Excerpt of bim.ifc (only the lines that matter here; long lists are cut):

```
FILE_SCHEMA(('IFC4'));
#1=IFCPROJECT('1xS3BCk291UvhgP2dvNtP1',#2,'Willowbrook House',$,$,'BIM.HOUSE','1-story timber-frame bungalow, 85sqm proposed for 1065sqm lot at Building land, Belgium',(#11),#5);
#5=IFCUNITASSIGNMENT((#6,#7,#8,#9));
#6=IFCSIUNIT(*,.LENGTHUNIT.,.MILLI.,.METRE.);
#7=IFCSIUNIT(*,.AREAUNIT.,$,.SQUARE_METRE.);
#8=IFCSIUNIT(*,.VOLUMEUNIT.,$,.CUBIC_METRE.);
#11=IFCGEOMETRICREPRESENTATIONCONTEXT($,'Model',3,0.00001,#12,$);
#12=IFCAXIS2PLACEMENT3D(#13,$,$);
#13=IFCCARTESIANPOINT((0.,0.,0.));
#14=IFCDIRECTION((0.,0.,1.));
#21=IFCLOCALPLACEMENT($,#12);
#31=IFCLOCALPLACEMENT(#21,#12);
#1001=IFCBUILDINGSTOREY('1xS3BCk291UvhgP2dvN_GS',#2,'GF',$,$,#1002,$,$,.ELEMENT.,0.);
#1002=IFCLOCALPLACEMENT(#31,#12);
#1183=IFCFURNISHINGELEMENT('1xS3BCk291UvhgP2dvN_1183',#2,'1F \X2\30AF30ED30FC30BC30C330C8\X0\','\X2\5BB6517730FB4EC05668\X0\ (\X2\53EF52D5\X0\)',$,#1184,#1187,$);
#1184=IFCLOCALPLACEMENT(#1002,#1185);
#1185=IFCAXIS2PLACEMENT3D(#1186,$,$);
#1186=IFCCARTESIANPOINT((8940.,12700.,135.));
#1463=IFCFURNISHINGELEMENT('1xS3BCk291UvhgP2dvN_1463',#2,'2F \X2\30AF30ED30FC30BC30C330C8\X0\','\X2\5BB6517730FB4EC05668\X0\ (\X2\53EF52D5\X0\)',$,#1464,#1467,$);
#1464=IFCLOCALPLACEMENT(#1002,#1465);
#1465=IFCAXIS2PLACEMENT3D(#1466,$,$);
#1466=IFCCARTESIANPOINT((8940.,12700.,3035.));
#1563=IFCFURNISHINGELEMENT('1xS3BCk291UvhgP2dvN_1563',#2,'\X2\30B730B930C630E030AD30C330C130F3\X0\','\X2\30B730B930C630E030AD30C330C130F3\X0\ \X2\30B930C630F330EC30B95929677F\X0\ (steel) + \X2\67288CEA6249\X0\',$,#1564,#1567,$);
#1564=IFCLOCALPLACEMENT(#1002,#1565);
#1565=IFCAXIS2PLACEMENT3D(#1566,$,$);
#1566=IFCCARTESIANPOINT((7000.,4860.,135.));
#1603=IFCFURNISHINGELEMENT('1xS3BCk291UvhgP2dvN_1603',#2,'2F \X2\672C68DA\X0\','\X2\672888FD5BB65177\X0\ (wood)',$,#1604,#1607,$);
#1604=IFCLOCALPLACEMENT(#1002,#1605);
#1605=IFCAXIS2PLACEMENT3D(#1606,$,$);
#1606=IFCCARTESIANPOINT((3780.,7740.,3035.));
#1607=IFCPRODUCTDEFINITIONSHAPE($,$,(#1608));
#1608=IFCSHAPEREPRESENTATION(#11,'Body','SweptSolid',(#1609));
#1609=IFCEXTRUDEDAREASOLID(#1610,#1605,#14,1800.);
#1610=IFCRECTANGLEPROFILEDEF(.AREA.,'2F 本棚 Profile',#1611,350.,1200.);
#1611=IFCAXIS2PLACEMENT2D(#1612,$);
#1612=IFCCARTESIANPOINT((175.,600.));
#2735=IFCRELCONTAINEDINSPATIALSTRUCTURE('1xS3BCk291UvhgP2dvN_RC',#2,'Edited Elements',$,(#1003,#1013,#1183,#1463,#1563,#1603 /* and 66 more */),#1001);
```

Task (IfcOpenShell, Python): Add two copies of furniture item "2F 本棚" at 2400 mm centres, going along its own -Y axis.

```python
import ifcopenshell
import ifcopenshell.api.geometry
import ifcopenshell.api.root
import ifcopenshell.util.element
import ifcopenshell.util.placement
import ifcopenshell.util.unit

model = ifcopenshell.open("bim.ifc")
unit_scale = ifcopenshell.util.unit.calculate_unit_scale(model)


def reuse_history(source, copy):
    """copy_class also copies each property set's owner history, people and application; keep the originals."""
    for rel in copy.IsDefinedBy:
        if rel.is_a("IfcRelDefinesByProperties") and (history := rel.RelatingPropertyDefinition.OwnerHistory):
            rel.RelatingPropertyDefinition.OwnerHistory = source.OwnerHistory
            ifcopenshell.util.element.remove_deep2(model, history)


source = model.by_guid("1xS3BCk291UvhgP2dvN_1603")
base = ifcopenshell.util.placement.get_local_placement(source.ObjectPlacement)
step = -base[:3, 1] * 2.4 / unit_scale

for i in range(1, 3):
    copy = ifcopenshell.api.root.copy_class(model, product=source)
    copy.Representation = ifcopenshell.util.element.copy_deep(
        model, source.Representation, exclude=["IfcGeometricRepresentationContext", "IfcRepresentationMap"]
    )
    reuse_history(source, copy)
    matrix = base.copy()
    matrix[:3, 3] += i * step
    print("added at", matrix[:3, 3].round(3) + 0.0)
    ifcopenshell.api.geometry.edit_object_placement(model, product=copy, matrix=matrix, is_si=False)

model.write("bim_edited.ifc")
```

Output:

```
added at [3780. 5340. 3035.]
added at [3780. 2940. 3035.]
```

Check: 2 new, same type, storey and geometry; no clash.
